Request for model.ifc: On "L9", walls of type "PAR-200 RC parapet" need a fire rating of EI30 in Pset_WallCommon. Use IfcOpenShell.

First a look at what the model holds.

```python
import ifcopenshell
import ifcopenshell.util.element

model = ifcopenshell.open("model.ifc")
print(model.schema)
storey = next(s for s in model.by_type("IfcBuildingStorey") if s.Name == "L9")
walls = [e for e in ifcopenshell.util.element.get_decomposition(storey) if e.is_a("IfcWall")]
seen = {}
for e in walls:
    element_type = ifcopenshell.util.element.get_type(e)
    key = (element_type.Name if element_type != e and element_type else None, ifcopenshell.util.element.get_pset(e, "Pset_WallCommon", "FireRating"))
    seen[key] = seen.get(key, 0) + 1
for (name, value), count in sorted(seen.items(), key=str):
    print(count, "x", name, "|", value)
```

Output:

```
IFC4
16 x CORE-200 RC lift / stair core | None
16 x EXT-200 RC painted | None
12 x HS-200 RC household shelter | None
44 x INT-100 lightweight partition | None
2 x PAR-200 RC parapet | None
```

```python
import ifcopenshell
import ifcopenshell.api.pset
import ifcopenshell.util.element

model = ifcopenshell.open("model.ifc")

storey = next(s for s in model.by_type("IfcBuildingStorey") if s.Name == "L9")
walls = [e for e in ifcopenshell.util.element.get_decomposition(storey) if e.is_a("IfcWall")]

count = 0
for e in walls:
    element_type = ifcopenshell.util.element.get_type(e)
    if element_type in (None, e) or element_type.Name != "PAR-200 RC parapet":
        continue
    # add_pset returns the element's existing set when there is one.
    pset = ifcopenshell.api.pset.add_pset(model, product=e, name="Pset_WallCommon")
    ifcopenshell.api.pset.edit_pset(model, pset=pset, properties={"FireRating": "EI30"})
    count += 1

print(count, "walls updated")

model.write("model-out.ifc")
```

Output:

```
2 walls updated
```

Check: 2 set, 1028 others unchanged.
